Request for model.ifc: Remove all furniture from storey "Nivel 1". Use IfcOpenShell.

First a look at what the model holds.

```python
import ifcopenshell
import ifcopenshell.util.element

model = ifcopenshell.open("model.ifc")
print(model.schema)
storey = next(s for s in model.by_type("IfcBuildingStorey") if s.Name == "Nivel 1")
furniture = [e for e in ifcopenshell.util.element.get_decomposition(storey) if e.is_a("IfcFurnishingElement")]
seen = {}
for e in furniture:
    element_type = ifcopenshell.util.element.get_type(e)
    name = element_type.Name if element_type not in (None, e) else None
    seen[name] = seen.get(name, 0) + 1
for name, count in sorted(seen.items(), key=str):
    print(count, "x", name)
```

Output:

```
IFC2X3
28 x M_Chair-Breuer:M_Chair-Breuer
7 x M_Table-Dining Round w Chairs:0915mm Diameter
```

```python
import ifcopenshell
import ifcopenshell.api.root
import ifcopenshell.util.element

model = ifcopenshell.open("model.ifc")

storey = next(s for s in model.by_type("IfcBuildingStorey") if s.Name == "Nivel 1")
furniture = [e for e in ifcopenshell.util.element.get_decomposition(storey) if e.is_a("IfcFurnishingElement")]

for e in furniture:
    ifcopenshell.api.root.remove_product(model, product=e)
print(len(furniture), "removed")

model.write("model_updated.ifc")
```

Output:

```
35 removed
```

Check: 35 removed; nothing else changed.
